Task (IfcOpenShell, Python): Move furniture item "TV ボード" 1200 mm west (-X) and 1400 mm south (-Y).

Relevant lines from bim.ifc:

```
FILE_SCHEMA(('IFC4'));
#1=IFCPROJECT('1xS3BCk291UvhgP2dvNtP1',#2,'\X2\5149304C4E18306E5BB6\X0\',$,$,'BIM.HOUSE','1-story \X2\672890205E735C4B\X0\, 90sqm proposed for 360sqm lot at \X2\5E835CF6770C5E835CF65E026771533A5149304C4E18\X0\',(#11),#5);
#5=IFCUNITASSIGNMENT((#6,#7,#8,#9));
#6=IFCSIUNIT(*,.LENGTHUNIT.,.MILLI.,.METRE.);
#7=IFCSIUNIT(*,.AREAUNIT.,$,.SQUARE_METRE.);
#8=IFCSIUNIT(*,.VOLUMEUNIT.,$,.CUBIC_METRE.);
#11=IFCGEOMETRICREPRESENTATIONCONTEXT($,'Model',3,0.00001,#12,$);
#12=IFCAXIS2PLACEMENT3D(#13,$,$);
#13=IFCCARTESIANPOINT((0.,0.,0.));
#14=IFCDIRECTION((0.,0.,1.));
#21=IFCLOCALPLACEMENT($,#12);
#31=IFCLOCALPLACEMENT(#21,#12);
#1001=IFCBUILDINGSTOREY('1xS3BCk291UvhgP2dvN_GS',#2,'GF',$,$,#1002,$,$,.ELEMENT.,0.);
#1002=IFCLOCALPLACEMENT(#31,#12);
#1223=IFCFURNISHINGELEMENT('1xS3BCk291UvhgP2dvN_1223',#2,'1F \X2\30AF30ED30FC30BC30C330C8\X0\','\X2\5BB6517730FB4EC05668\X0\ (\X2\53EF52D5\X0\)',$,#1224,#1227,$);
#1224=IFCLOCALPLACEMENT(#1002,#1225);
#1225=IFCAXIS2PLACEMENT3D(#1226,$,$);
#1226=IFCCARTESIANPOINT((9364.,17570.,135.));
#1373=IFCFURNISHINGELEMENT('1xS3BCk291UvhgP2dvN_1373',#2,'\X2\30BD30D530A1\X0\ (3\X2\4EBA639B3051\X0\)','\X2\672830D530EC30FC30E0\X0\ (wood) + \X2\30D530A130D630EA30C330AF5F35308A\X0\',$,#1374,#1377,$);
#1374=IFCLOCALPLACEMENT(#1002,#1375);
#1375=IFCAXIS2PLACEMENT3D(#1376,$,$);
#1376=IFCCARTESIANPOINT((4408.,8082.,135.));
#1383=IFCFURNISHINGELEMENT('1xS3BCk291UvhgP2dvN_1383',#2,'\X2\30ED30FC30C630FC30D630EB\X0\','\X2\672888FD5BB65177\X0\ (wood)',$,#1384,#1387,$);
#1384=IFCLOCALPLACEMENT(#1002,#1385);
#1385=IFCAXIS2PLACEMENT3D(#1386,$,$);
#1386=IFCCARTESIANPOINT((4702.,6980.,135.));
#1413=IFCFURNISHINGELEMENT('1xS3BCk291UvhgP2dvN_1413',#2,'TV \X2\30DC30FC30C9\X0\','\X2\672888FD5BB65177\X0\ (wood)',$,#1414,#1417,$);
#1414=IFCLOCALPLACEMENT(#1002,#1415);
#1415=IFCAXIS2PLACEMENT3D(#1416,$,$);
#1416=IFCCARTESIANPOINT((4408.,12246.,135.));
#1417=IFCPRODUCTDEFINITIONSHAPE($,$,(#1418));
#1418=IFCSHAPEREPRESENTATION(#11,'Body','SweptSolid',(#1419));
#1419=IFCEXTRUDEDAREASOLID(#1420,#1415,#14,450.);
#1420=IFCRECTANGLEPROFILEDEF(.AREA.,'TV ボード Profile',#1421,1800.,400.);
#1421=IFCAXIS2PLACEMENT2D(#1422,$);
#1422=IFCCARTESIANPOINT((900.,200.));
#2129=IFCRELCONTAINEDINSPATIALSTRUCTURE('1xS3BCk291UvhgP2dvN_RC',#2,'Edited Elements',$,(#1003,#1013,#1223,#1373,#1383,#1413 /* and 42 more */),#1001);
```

```python
import ifcopenshell
import ifcopenshell.api.geometry
import ifcopenshell.util.placement
import ifcopenshell.util.unit

model = ifcopenshell.open("bim.ifc")
unit_scale = ifcopenshell.util.unit.calculate_unit_scale(model)

item = model.by_guid("1xS3BCk291UvhgP2dvN_1413")
matrix = ifcopenshell.util.placement.get_local_placement(item.ObjectPlacement)
matrix[0, 3] -= 1.2 / unit_scale
matrix[1, 3] -= 1.4 / unit_scale
ifcopenshell.api.geometry.edit_object_placement(model, product=item, matrix=matrix, is_si=False)

print(ifcopenshell.util.placement.get_local_placement(item.ObjectPlacement).round(3) + 0.0)

model.write("bim_rev.ifc")
```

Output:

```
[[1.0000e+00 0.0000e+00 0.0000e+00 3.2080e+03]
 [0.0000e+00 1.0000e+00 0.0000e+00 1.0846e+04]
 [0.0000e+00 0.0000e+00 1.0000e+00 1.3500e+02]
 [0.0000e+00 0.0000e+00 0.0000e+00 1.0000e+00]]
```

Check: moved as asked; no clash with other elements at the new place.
